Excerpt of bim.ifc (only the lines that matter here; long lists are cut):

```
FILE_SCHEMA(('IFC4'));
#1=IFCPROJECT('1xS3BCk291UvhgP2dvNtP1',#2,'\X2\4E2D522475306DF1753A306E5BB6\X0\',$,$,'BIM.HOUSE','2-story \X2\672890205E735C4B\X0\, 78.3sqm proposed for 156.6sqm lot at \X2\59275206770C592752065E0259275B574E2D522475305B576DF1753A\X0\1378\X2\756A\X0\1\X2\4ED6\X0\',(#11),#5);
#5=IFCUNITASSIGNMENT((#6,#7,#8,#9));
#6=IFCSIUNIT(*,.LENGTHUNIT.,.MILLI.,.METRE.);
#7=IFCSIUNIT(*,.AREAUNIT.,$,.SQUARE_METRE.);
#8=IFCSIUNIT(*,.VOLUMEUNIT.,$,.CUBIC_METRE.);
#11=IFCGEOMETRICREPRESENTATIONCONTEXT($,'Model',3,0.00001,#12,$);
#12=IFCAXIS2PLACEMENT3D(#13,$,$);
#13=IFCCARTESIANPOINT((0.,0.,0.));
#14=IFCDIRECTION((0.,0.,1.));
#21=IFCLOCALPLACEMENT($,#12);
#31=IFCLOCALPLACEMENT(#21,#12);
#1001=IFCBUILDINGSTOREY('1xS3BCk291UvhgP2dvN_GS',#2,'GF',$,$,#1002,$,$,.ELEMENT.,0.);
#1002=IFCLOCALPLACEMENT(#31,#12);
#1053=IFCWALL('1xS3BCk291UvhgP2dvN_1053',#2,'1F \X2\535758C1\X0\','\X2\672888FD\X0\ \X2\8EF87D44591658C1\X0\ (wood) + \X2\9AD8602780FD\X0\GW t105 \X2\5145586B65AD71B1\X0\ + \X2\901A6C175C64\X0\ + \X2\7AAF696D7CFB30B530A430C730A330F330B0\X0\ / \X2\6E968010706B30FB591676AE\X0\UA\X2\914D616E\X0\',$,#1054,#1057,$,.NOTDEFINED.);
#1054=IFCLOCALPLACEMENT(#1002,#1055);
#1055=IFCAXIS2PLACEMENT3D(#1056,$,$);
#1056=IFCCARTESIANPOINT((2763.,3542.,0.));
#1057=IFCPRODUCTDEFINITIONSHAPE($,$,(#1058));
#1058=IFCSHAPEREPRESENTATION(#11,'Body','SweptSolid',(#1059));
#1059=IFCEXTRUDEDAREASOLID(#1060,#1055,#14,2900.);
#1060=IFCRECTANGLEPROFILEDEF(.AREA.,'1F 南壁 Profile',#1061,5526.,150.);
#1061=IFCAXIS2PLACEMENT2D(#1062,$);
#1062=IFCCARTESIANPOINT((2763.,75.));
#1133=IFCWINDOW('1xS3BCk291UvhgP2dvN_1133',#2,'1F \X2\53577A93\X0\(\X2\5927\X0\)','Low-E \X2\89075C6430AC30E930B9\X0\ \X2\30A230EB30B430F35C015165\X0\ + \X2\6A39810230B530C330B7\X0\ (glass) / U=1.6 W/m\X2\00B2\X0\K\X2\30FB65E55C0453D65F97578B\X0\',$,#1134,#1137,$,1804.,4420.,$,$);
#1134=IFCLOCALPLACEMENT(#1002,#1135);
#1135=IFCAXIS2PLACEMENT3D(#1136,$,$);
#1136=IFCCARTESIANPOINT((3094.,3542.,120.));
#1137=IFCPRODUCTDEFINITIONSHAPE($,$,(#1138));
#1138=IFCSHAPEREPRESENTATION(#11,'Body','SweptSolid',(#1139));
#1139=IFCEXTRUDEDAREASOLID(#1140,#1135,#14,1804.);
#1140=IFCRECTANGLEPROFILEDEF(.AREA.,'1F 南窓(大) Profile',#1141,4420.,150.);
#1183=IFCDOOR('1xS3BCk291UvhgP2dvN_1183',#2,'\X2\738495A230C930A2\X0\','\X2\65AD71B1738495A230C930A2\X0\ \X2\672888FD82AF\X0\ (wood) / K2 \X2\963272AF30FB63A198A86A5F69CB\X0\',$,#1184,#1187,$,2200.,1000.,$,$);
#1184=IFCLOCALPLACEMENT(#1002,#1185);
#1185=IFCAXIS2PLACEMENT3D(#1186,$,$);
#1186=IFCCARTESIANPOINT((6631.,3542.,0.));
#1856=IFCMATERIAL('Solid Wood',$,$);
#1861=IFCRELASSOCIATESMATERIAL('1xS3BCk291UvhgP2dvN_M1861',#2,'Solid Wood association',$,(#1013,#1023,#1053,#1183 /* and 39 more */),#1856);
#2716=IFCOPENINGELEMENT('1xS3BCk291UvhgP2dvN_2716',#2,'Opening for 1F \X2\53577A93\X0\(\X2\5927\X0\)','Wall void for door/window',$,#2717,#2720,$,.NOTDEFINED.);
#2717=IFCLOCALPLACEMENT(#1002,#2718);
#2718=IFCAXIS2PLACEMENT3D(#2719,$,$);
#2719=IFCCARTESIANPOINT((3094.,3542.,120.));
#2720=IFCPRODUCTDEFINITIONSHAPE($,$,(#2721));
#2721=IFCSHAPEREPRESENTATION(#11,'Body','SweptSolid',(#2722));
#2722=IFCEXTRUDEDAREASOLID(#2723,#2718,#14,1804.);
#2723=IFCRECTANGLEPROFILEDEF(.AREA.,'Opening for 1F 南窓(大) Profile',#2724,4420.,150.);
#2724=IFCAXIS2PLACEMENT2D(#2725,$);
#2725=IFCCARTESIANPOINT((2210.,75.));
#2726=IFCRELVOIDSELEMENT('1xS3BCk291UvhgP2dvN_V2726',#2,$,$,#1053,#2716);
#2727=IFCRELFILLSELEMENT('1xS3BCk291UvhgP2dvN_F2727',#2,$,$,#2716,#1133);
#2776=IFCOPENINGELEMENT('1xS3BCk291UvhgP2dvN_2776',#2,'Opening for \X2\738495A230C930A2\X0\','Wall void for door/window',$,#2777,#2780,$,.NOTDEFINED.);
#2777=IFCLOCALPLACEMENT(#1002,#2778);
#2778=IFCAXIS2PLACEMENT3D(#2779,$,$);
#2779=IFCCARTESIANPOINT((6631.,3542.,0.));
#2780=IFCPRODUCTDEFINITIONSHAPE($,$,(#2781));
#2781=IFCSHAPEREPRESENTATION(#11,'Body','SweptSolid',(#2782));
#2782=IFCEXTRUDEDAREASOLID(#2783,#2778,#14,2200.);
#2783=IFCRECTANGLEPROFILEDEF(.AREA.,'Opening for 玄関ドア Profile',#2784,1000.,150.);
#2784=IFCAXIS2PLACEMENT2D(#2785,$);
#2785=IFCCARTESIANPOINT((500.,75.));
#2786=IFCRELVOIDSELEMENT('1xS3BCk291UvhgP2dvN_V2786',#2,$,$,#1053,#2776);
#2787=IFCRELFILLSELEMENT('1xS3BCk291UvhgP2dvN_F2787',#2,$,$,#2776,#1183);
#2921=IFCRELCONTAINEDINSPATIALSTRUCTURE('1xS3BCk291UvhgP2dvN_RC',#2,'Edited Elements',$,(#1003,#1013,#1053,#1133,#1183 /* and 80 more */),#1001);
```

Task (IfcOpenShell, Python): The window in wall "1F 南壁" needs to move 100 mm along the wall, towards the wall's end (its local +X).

```python
import ifcopenshell
import ifcopenshell.api.geometry
import ifcopenshell.util.placement
import ifcopenshell.util.unit

model = ifcopenshell.open("bim.ifc")
unit_scale = ifcopenshell.util.unit.calculate_unit_scale(model)

window = model.by_guid("1xS3BCk291UvhgP2dvN_1133")
opening = window.FillsVoids[0].RelatingOpeningElement
wall = opening.VoidsElements[0].RelatingBuildingElement

wall_matrix = ifcopenshell.util.placement.get_local_placement(wall.ObjectPlacement)
shift = wall_matrix[:3, 0] * 0.1 / unit_scale
before = ifcopenshell.util.placement.get_local_placement(window.ObjectPlacement)[:3, 3].copy()

# The window is not placed relative to its opening, so move both.
for product in (opening, window):
    matrix = ifcopenshell.util.placement.get_local_placement(product.ObjectPlacement)
    matrix[:3, 3] += shift
    ifcopenshell.api.geometry.edit_object_placement(model, product=product, matrix=matrix, is_si=False)

after = ifcopenshell.util.placement.get_local_placement(window.ObjectPlacement)[:3, 3]
print("window moved by", (after - before).round(3) + 0.0)

model.write("bim_edited.ifc")
```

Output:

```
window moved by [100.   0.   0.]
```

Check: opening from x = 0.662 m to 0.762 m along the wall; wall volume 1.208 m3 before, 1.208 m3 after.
